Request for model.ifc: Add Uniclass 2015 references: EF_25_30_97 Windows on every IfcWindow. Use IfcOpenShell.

First a look at what the model holds.

```python
import ifcopenshell

model = ifcopenshell.open("model.ifc")
print(model.schema)
print("classifications:", [c.Name for c in model.by_type("IfcClassification")])
for ifc_class in ("IfcDoor", "IfcRoof", "IfcStair", "IfcWall", "IfcWindow"):
    print(ifc_class, len(model.by_type(ifc_class)))
```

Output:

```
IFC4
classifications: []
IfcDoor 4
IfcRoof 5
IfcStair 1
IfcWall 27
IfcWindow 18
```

```python
import ifcopenshell
import ifcopenshell.api.classification

model = ifcopenshell.open("model.ifc")

system = ifcopenshell.api.classification.add_classification(model, classification="Uniclass 2015")

codes = {
    "IfcWindow": ("EF_25_30_97", "Windows"),
}
for ifc_class, (code, name) in codes.items():
    products = model.by_type(ifc_class)
    ifcopenshell.api.classification.add_reference(
        model, products=products, classification=system, identification=code, name=name
    )
    print(code, len(products))

model.write("model_edited.ifc")
```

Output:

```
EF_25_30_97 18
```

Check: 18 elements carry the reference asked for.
